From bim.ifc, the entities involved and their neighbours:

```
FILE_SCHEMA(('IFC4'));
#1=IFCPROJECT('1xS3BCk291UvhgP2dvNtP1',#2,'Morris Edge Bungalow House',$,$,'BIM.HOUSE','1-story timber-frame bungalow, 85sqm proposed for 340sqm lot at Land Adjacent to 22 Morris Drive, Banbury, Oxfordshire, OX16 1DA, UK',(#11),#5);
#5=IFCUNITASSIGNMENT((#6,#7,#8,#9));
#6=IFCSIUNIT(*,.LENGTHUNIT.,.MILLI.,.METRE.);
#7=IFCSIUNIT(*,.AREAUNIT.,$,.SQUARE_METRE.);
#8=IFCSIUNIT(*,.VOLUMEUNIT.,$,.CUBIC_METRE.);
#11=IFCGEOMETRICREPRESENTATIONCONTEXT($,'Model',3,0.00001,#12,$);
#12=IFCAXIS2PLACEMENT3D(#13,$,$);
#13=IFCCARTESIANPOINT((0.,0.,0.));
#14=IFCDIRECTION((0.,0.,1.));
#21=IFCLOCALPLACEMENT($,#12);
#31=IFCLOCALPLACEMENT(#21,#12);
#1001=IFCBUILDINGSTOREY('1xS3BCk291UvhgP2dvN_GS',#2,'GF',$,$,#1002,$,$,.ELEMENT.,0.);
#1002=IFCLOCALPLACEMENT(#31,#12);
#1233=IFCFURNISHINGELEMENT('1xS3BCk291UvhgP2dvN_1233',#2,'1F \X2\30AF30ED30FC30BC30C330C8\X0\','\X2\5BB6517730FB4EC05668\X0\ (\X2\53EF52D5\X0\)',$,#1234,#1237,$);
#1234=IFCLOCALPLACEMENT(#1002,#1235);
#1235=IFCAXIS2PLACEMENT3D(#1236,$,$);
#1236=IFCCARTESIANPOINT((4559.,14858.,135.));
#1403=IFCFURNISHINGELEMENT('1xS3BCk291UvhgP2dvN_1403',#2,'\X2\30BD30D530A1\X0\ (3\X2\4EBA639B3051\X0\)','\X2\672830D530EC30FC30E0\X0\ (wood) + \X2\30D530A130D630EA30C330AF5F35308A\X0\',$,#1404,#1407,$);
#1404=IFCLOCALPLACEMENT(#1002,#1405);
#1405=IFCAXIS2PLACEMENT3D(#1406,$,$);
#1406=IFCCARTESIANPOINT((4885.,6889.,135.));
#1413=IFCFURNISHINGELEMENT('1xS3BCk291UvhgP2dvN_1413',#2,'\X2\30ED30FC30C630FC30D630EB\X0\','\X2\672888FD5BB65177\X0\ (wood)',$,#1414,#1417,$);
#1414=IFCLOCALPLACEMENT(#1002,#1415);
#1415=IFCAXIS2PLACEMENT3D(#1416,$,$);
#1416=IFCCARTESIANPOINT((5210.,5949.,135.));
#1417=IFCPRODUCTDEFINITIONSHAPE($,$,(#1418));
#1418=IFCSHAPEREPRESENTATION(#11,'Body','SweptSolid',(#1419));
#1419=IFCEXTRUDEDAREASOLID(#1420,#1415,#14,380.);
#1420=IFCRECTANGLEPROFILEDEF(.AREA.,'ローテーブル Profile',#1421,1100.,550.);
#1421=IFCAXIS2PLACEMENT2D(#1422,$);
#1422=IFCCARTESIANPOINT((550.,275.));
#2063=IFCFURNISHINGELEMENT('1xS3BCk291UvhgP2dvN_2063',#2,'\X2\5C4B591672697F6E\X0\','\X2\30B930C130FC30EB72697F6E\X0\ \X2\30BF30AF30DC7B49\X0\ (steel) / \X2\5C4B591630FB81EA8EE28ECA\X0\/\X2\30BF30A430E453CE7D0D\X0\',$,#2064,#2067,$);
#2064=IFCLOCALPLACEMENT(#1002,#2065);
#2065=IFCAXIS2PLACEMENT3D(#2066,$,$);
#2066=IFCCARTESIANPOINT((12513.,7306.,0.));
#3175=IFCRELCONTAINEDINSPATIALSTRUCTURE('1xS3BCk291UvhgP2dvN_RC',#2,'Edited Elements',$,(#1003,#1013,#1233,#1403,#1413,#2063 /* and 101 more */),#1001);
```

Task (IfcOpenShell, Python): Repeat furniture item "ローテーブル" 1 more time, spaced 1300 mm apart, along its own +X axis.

```python
import ifcopenshell
import ifcopenshell.api.geometry
import ifcopenshell.api.root
import ifcopenshell.util.element
import ifcopenshell.util.placement

model = ifcopenshell.open("bim.ifc")


def reuse_history(source, copy):
    """copy_class also copies each property set's owner history, people and application; keep the originals."""
    for rel in copy.IsDefinedBy:
        if rel.is_a("IfcRelDefinesByProperties") and (history := rel.RelatingPropertyDefinition.OwnerHistory):
            rel.RelatingPropertyDefinition.OwnerHistory = source.OwnerHistory
            ifcopenshell.util.element.remove_deep2(model, history)


source = model.by_guid("1xS3BCk291UvhgP2dvN_1413")
base = ifcopenshell.util.placement.get_local_placement(source.ObjectPlacement)
step = base[:3, 0] * 1300.0

for i in range(1, 2):
    copy = ifcopenshell.api.root.copy_class(model, product=source)
    copy.Representation = ifcopenshell.util.element.copy_deep(
        model, source.Representation, exclude=["IfcGeometricRepresentationContext", "IfcRepresentationMap"]
    )
    reuse_history(source, copy)
    matrix = base.copy()
    matrix[:3, 3] += i * step
    print("added at", matrix[:3, 3].round(3) + 0.0)
    ifcopenshell.api.geometry.edit_object_placement(model, product=copy, matrix=matrix, is_si=False)

model.write("bim-out.ifc")
```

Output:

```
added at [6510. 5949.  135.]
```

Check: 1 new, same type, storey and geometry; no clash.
